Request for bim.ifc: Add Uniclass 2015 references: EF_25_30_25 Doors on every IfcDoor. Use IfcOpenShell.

First a look at what the model holds.

```python
import ifcopenshell

model = ifcopenshell.open("bim.ifc")
print(model.schema)
print("classifications:", [c.Name for c in model.by_type("IfcClassification")])
for ifc_class in ("IfcDoor", "IfcRoof", "IfcStair", "IfcWall", "IfcWindow"):
    print(ifc_class, len(model.by_type(ifc_class)))
```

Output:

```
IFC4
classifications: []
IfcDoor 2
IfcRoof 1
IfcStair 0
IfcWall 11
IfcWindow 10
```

```python
import ifcopenshell
import ifcopenshell.api.classification

model = ifcopenshell.open("bim.ifc")

system = ifcopenshell.api.classification.add_classification(model, classification="Uniclass 2015")

codes = {
    "IfcDoor": ("EF_25_30_25", "Doors"),
}
for ifc_class, (code, name) in codes.items():
    products = model.by_type(ifc_class)
    ifcopenshell.api.classification.add_reference(
        model, products=products, classification=system, identification=code, name=name
    )
    print(code, len(products))

model.write("bim_updated.ifc")
```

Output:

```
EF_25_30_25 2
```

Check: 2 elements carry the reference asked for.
